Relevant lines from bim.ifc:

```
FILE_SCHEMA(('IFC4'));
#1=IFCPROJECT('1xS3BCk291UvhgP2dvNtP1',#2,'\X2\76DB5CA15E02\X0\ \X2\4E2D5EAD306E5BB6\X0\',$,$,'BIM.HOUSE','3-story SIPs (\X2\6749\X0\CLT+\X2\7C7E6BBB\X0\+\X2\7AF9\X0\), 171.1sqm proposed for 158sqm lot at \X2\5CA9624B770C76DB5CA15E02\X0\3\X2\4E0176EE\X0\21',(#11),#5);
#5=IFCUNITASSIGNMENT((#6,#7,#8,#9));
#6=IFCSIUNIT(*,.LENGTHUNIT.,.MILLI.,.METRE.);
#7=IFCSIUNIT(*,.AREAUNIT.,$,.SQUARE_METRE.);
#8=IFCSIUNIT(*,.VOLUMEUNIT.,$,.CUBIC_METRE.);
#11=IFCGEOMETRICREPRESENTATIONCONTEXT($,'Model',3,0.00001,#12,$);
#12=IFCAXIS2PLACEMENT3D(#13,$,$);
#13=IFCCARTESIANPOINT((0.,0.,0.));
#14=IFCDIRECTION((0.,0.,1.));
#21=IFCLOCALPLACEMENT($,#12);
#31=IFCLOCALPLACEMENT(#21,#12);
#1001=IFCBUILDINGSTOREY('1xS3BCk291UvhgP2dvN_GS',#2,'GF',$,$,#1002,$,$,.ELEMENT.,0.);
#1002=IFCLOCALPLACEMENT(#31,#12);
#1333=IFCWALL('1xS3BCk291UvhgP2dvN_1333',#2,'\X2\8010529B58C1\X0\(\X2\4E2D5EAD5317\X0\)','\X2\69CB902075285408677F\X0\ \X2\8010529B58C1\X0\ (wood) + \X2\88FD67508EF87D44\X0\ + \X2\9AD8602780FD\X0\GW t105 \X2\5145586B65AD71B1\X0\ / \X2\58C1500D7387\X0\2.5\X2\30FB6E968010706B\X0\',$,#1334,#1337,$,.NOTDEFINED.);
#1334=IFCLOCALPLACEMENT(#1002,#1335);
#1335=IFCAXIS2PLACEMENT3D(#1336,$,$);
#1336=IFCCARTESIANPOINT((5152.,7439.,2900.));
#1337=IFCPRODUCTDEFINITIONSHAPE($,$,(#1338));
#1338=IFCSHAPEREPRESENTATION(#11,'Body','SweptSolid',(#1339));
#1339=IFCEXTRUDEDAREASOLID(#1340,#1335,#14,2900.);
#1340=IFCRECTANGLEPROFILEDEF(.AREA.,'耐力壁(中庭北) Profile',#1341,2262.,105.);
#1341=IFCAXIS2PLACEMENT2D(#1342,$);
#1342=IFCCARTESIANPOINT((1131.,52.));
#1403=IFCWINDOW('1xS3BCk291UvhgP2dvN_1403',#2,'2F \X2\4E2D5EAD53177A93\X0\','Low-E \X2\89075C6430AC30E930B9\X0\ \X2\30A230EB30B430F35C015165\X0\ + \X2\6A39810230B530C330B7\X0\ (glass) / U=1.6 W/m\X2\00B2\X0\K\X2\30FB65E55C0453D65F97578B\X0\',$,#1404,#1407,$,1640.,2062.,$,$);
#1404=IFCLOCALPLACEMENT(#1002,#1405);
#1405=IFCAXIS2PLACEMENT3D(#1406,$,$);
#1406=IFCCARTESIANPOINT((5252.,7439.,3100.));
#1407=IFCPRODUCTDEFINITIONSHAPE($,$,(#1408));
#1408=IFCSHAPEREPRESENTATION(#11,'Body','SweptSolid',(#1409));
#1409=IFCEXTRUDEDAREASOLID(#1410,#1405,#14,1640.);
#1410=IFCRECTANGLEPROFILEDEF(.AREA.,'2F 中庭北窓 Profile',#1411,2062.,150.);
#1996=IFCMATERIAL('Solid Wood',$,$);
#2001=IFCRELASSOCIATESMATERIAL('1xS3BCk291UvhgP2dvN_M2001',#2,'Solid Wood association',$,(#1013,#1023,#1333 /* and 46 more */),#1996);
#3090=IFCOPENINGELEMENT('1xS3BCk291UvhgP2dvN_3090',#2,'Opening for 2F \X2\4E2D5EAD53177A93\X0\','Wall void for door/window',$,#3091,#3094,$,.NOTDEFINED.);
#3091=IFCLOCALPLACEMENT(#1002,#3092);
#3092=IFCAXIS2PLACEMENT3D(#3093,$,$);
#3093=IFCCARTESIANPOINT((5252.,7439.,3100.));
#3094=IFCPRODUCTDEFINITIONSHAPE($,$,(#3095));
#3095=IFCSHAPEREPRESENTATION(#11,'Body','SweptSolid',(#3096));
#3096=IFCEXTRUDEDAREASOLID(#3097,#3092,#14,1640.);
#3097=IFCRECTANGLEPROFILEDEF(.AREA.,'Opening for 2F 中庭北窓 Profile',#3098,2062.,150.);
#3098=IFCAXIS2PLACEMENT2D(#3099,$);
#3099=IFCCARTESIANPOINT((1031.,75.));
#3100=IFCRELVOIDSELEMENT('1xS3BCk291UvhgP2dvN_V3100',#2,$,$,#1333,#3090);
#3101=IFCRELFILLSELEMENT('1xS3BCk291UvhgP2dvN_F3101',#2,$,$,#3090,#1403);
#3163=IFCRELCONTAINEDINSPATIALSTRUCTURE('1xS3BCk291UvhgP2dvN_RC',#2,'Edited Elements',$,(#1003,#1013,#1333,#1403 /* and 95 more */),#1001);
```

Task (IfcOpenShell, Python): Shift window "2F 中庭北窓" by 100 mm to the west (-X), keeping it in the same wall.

```python
import ifcopenshell
import ifcopenshell.api.geometry
import ifcopenshell.util.placement

model = ifcopenshell.open("bim.ifc")

window = model.by_guid("1xS3BCk291UvhgP2dvN_1403")
opening = window.FillsVoids[0].RelatingOpeningElement
wall = opening.VoidsElements[0].RelatingBuildingElement

wall_matrix = ifcopenshell.util.placement.get_local_placement(wall.ObjectPlacement)
shift = wall_matrix[:3, 0] * -100.0
before = ifcopenshell.util.placement.get_local_placement(window.ObjectPlacement)[:3, 3].copy()

# The window is not placed relative to its opening, so move both.
for product in (opening, window):
    matrix = ifcopenshell.util.placement.get_local_placement(product.ObjectPlacement)
    matrix[:3, 3] += shift
    ifcopenshell.api.geometry.edit_object_placement(model, product=product, matrix=matrix, is_si=False)

after = ifcopenshell.util.placement.get_local_placement(window.ObjectPlacement)[:3, 3]
print("window moved by", (after - before).round(3) + 0.0)

model.write("bim_rev.ifc")
```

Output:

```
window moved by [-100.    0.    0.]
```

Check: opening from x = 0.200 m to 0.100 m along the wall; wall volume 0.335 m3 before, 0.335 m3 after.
